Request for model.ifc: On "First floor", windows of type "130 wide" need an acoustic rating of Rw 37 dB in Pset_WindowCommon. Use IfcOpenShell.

First a look at what the model holds.

```python
import ifcopenshell
import ifcopenshell.util.element

model = ifcopenshell.open("model.ifc")
print(model.schema)
storey = next(s for s in model.by_type("IfcBuildingStorey") if s.Name == "First floor")
windows = [e for e in ifcopenshell.util.element.get_decomposition(storey) if e.is_a("IfcWindow")]
seen = {}
for e in windows:
    element_type = ifcopenshell.util.element.get_type(e)
    key = (element_type.Name if element_type != e and element_type else None, ifcopenshell.util.element.get_pset(e, "Pset_WindowCommon", "AcousticRating"))
    seen[key] = seen.get(key, 0) + 1
for (name, value), count in sorted(seen.items(), key=str):
    print(count, "x", name, "|", value)
```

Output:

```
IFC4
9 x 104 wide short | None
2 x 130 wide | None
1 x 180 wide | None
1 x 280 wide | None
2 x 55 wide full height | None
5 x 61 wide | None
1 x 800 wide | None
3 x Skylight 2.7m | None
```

```python
import ifcopenshell
import ifcopenshell.api.pset
import ifcopenshell.util.element

model = ifcopenshell.open("model.ifc")

storey = next(s for s in model.by_type("IfcBuildingStorey") if s.Name == "First floor")
windows = [e for e in ifcopenshell.util.element.get_decomposition(storey) if e.is_a("IfcWindow")]

count = 0
for e in windows:
    element_type = ifcopenshell.util.element.get_type(e)
    if element_type in (None, e) or element_type.Name != "130 wide":
        continue
    # add_pset returns the element's existing set when there is one.
    pset = ifcopenshell.api.pset.add_pset(model, product=e, name="Pset_WindowCommon")
    ifcopenshell.api.pset.edit_pset(model, pset=pset, properties={"AcousticRating": "Rw 37 dB"})
    count += 1

print(count, "windows updated")

model.write("model-out.ifc")
```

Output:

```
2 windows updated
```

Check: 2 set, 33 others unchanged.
